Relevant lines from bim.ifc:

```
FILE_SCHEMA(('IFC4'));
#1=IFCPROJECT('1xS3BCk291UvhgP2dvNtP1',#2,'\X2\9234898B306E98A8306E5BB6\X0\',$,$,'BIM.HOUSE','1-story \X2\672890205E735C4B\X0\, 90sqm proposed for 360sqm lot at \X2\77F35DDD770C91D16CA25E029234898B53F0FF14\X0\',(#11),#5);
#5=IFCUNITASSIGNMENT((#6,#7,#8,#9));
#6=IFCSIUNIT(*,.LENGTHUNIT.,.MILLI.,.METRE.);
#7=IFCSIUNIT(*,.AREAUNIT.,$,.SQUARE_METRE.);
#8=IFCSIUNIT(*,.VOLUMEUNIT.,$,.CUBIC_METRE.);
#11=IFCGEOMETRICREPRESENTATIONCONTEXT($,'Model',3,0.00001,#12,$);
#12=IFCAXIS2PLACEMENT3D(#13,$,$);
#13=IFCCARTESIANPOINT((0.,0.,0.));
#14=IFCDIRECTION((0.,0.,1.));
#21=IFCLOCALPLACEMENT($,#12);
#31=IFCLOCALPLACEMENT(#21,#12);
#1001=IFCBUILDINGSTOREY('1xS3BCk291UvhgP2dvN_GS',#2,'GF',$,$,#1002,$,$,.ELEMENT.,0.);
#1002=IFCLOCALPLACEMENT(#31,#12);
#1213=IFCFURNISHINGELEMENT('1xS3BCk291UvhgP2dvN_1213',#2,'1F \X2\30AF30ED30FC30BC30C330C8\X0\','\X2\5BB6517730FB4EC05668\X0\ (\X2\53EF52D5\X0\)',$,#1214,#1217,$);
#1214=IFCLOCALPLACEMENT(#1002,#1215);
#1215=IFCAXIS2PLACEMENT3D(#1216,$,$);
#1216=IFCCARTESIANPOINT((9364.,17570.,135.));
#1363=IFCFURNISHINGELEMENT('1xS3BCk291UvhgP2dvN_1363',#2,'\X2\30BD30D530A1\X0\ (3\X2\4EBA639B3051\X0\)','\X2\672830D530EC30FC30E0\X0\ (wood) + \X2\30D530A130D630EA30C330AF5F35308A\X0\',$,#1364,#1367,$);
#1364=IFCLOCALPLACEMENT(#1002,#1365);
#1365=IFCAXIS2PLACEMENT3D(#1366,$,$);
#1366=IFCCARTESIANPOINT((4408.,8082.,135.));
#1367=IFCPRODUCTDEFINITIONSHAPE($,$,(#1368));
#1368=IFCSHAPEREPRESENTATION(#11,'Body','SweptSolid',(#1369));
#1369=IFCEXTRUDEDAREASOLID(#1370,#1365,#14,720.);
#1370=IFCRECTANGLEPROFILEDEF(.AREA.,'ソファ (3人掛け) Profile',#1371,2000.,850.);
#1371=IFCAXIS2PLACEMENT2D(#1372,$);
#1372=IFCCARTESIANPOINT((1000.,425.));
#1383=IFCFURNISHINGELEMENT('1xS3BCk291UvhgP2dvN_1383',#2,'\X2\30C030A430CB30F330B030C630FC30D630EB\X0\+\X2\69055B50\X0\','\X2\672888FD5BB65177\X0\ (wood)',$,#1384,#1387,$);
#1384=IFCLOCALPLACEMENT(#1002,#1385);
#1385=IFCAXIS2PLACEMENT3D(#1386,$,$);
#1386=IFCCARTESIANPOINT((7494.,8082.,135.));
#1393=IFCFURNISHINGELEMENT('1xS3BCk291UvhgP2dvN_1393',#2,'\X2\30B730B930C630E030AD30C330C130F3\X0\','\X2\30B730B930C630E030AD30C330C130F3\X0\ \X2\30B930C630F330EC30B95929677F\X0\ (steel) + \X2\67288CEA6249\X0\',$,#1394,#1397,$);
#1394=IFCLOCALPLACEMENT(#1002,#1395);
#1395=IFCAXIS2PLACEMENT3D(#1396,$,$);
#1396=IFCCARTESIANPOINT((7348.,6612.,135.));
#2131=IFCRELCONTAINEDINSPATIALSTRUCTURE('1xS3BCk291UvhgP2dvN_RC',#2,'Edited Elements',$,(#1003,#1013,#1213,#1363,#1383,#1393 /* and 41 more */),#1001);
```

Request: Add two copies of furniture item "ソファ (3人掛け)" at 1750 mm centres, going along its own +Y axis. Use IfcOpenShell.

```python
import ifcopenshell
import ifcopenshell.api.geometry
import ifcopenshell.api.root
import ifcopenshell.util.element
import ifcopenshell.util.placement

model = ifcopenshell.open("bim.ifc")


def reuse_history(source, copy):
    """copy_class also copies each property set's owner history, people and application; keep the originals."""
    for rel in copy.IsDefinedBy:
        if rel.is_a("IfcRelDefinesByProperties") and (history := rel.RelatingPropertyDefinition.OwnerHistory):
            rel.RelatingPropertyDefinition.OwnerHistory = source.OwnerHistory
            ifcopenshell.util.element.remove_deep2(model, history)


source = model.by_guid("1xS3BCk291UvhgP2dvN_1363")
base = ifcopenshell.util.placement.get_local_placement(source.ObjectPlacement)
step = base[:3, 1] * 1750.0

for i in range(1, 3):
    copy = ifcopenshell.api.root.copy_class(model, product=source)
    copy.Representation = ifcopenshell.util.element.copy_deep(
        model, source.Representation, exclude=["IfcGeometricRepresentationContext", "IfcRepresentationMap"]
    )
    reuse_history(source, copy)
    matrix = base.copy()
    matrix[:3, 3] += i * step
    print("added at", matrix[:3, 3].round(3) + 0.0)
    ifcopenshell.api.geometry.edit_object_placement(model, product=copy, matrix=matrix, is_si=False)

model.write("bim_rev.ifc")
```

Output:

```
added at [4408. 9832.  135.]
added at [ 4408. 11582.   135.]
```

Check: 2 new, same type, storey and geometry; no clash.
